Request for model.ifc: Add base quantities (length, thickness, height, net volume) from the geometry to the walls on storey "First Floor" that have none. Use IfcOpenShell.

First a look at what the model holds.

```python
import ifcopenshell
import ifcopenshell.util.element
import ifcopenshell.util.unit

model = ifcopenshell.open("model.ifc")
print(model.schema)
for unit_type in ("LENGTHUNIT", "AREAUNIT", "VOLUMEUNIT"):
    print(unit_type, ifcopenshell.util.unit.calculate_unit_scale(model, unit_type))
storey = next(s for s in model.by_type("IfcBuildingStorey") if s.Name == "First Floor")
walls = [e for e in ifcopenshell.util.element.get_decomposition(storey) if e.is_a("IfcWall")]
for e in sorted(walls, key=lambda e: e.id()):
    print(e.id(), e.is_a(), e.Name, list(ifcopenshell.util.element.get_psets(e, qtos_only=True)), sep=" | ")
```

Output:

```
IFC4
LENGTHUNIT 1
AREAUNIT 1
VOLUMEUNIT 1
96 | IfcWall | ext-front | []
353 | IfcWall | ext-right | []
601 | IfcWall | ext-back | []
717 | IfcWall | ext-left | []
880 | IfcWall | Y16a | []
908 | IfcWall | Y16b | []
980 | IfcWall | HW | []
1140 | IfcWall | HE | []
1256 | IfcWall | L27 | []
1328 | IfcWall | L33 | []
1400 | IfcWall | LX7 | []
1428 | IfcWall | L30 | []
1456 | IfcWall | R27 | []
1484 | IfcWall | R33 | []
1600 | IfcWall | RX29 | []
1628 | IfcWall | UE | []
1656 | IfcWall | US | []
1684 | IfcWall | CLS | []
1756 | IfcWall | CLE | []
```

```python
import ifcopenshell
import ifcopenshell.api.pset
import ifcopenshell.geom
import ifcopenshell.util.element
import ifcopenshell.util.shape
import ifcopenshell.util.unit

model = ifcopenshell.open("model.ifc")
unit_scale = ifcopenshell.util.unit.calculate_unit_scale(model)
volume_scale = ifcopenshell.util.unit.calculate_unit_scale(model, "VOLUMEUNIT")
settings = ifcopenshell.geom.settings()

storey = next(s for s in model.by_type("IfcBuildingStorey") if s.Name == "First Floor")
walls = [e for e in ifcopenshell.util.element.get_decomposition(storey) if e.is_a("IfcWall")]

for e in sorted(walls, key=lambda e: e.id()):
    if ifcopenshell.util.element.get_psets(e, qtos_only=True, should_inherit=False):
        continue
    # Geometry comes back in metres, in the element's own axes.
    shape = ifcopenshell.geom.create_shape(settings, e)
    values = {
        "Length": ifcopenshell.util.shape.get_x(shape.geometry) / unit_scale,
        "Width": ifcopenshell.util.shape.get_y(shape.geometry) / unit_scale,
        "Height": ifcopenshell.util.shape.get_z(shape.geometry) / unit_scale,
        "NetVolume": ifcopenshell.util.shape.get_volume(shape.geometry) / volume_scale,
    }
    qto = ifcopenshell.api.pset.add_qto(model, product=e, name="Qto_WallBaseQuantities")
    ifcopenshell.api.pset.edit_qto(model, qto=qto, properties=values)
    print(e.id(), {k: round(v, 3) for k, v in values.items()})

model.write("model_v2.ifc")
```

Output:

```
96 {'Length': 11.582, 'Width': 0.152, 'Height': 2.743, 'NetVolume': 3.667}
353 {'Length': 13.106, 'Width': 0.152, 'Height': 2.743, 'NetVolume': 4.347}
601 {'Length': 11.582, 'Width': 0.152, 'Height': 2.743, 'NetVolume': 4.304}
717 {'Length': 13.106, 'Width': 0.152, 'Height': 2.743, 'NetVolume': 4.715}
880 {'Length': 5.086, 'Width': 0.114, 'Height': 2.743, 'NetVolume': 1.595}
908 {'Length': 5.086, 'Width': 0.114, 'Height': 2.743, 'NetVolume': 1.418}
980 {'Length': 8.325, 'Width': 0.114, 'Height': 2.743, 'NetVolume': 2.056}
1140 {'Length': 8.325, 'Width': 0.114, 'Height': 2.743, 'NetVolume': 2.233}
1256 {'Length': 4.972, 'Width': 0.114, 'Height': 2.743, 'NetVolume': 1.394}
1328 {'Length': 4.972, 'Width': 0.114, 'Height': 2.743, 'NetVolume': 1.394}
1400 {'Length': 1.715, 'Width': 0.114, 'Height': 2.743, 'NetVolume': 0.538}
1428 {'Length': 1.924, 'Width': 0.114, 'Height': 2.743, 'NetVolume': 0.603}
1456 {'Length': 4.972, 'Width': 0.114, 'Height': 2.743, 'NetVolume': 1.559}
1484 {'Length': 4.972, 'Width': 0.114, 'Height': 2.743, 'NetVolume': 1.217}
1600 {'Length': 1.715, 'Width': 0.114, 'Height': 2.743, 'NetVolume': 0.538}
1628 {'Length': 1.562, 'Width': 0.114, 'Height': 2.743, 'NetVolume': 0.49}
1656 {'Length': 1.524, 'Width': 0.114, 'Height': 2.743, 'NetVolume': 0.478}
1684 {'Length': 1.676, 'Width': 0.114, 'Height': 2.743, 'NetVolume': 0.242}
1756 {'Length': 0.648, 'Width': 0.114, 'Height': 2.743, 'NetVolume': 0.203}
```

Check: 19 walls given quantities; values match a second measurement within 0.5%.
